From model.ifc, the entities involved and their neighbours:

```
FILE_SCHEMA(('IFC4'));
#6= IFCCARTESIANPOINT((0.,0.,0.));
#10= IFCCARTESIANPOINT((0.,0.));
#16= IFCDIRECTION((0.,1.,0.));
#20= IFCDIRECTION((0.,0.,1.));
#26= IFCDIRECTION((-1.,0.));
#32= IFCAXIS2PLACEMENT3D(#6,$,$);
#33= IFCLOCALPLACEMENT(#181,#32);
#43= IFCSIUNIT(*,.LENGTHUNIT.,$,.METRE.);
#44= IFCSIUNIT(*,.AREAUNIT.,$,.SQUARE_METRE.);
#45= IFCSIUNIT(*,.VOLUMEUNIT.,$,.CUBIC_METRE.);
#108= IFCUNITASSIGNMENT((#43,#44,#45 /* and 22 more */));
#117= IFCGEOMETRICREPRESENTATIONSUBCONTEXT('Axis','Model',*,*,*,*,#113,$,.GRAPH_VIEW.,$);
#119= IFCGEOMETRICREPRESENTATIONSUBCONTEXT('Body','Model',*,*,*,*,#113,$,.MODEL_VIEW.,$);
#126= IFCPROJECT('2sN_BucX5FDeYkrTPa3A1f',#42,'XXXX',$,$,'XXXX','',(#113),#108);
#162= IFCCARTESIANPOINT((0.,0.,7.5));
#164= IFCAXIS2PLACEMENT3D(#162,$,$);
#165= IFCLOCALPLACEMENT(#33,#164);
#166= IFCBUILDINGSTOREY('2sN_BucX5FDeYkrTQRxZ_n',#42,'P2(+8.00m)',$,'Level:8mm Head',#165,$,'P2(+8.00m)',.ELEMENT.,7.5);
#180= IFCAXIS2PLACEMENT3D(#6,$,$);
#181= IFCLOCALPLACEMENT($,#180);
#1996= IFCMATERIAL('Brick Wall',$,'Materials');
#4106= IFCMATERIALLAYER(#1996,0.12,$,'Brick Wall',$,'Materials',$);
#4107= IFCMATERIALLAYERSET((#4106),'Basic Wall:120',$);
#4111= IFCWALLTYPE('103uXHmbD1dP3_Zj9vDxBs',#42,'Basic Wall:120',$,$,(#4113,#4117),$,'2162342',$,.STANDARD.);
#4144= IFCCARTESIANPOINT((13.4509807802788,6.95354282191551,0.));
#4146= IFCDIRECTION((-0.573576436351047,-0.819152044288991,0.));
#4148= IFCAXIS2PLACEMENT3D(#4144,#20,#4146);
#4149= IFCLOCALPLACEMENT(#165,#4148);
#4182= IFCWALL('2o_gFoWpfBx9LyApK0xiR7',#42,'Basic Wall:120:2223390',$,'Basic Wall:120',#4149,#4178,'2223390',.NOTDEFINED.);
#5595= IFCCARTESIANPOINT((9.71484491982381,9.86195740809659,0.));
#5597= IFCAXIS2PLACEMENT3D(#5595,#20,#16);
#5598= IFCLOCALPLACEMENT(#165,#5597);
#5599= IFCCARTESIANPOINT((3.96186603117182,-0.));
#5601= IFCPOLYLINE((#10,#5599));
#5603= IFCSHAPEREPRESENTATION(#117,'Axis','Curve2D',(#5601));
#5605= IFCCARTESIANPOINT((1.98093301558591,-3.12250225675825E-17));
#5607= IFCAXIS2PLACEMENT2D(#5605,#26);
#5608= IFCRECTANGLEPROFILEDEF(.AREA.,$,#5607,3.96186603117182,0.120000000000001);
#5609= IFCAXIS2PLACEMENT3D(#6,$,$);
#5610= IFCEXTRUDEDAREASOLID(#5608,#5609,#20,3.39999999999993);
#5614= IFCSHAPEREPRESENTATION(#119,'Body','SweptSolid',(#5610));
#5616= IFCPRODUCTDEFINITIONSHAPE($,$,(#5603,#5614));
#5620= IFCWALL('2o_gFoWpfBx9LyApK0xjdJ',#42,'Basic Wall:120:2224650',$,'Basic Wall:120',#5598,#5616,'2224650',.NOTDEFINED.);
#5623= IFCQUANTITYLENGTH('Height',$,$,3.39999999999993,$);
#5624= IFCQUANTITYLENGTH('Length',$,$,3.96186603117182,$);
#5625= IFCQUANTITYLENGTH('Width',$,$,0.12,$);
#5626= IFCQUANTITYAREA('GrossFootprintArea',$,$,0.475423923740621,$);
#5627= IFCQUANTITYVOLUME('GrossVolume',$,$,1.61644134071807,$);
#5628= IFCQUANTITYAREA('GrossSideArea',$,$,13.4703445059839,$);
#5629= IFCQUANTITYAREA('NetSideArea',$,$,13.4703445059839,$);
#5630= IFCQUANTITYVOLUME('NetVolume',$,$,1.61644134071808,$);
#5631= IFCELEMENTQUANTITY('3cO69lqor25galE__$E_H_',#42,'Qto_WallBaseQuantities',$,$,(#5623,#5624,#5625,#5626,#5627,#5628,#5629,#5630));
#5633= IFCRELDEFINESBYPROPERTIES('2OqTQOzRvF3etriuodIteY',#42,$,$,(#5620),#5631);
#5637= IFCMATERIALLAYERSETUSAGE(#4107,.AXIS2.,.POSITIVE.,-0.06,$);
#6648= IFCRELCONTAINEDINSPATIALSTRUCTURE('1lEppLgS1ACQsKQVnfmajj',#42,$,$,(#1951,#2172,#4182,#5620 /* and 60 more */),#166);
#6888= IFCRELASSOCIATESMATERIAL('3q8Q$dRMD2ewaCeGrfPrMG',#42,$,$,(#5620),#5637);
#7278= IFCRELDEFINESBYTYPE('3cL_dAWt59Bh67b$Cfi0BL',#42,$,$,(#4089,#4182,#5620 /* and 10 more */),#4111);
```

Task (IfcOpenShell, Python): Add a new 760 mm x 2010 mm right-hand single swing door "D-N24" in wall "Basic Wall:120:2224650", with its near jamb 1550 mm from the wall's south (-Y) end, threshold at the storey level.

```python
import numpy as np
import ifcopenshell
import ifcopenshell.api.feature
import ifcopenshell.api.geometry
import ifcopenshell.api.pset
import ifcopenshell.api.root
import ifcopenshell.api.spatial
import ifcopenshell.geom
import ifcopenshell.util.element
import ifcopenshell.util.placement
import ifcopenshell.util.representation
import ifcopenshell.util.shape
import ifcopenshell.util.unit

model = ifcopenshell.open("model.ifc")
unit_scale = ifcopenshell.util.unit.calculate_unit_scale(model)
area_scale = ifcopenshell.util.unit.calculate_unit_scale(model, "AREAUNIT")
volume_scale = ifcopenshell.util.unit.calculate_unit_scale(model, "VOLUMEUNIT")
settings = ifcopenshell.geom.settings()


def volume(element):
    """Net volume in cubic metres, openings subtracted."""
    shape = ifcopenshell.geom.create_shape(settings, element)
    return ifcopenshell.util.shape.get_volume(shape.geometry)


wall = model.by_id(5620)
storey = ifcopenshell.util.element.get_container(wall, ifc_class="IfcBuildingStorey")
context = ifcopenshell.util.representation.get_context(model, "Model", "Body", "MODEL_VIEW")
before = volume(wall)

width, height, from_end, sill = 0.76, 2.01, 1.55, 0.0  # metres

# The wall runs along its own X axis, and the end named is its -X end.
wall_shape = ifcopenshell.geom.create_shape(settings, wall)
x, y, z = ifcopenshell.util.shape.get_vertices(wall_shape.geometry).T
start = x.min() + from_end
face, thickness = float(y.min()), float(y.max() - y.min())
wall_matrix = ifcopenshell.util.placement.get_local_placement(wall.ObjectPlacement)
level = ifcopenshell.util.placement.get_local_placement(storey.ObjectPlacement)[2, 3]


def in_wall(x, y):
    """Placement at x, y metres in the wall's axes, at sill height."""
    matrix = wall_matrix.copy()
    matrix[:, 3] = wall_matrix @ np.array([x / unit_scale, y / unit_scale, 0.0, 1.0])
    matrix[2, 3] = level + sill / unit_scale
    return matrix


# Opening: a box that overshoots both wall faces by 50 mm.
opening = ifcopenshell.api.root.create_entity(model, ifc_class="IfcOpeningElement", predefined_type="OPENING")
box = ifcopenshell.api.geometry.add_wall_representation(
    model, context=context, length=width, height=height, thickness=thickness + 0.1
)
ifcopenshell.api.geometry.assign_representation(model, product=opening, representation=box)
ifcopenshell.api.geometry.edit_object_placement(model, product=opening, matrix=in_wall(start, face - 0.05), is_si=False)
ifcopenshell.api.feature.add_feature(model, feature=opening, element=wall)

door = ifcopenshell.api.root.create_entity(model, ifc_class="IfcDoor", name="D-N24", predefined_type="DOOR")
door.OverallWidth, door.OverallHeight = width / unit_scale, height / unit_scale
door.OperationType = "SINGLE_SWING_RIGHT"
body = ifcopenshell.api.geometry.add_door_representation(
    model,
    context=context,
    overall_width=door.OverallWidth,
    overall_height=door.OverallHeight,
    operation_type="SINGLE_SWING_RIGHT",
    lining_properties={"LiningDepth": thickness / unit_scale, "ThresholdDepth": thickness / unit_scale},
)
ifcopenshell.api.geometry.assign_representation(model, product=door, representation=body)
ifcopenshell.api.spatial.assign_container(model, products=[door], relating_structure=storey)
ifcopenshell.api.feature.add_filling(model, opening=opening, element=door)

# The lining spans the wall, so the door starts at the wall face.
ifcopenshell.api.geometry.edit_object_placement(model, product=door, matrix=in_wall(start, face), is_si=False)

after = volume(wall)

# Update the wall's stored quantities.
qto = model.by_id(ifcopenshell.util.element.get_pset(wall, "Qto_WallBaseQuantities", should_inherit=False)["id"])
ifcopenshell.api.pset.edit_qto(model, qto=qto, properties={
    "NetSideArea": after / thickness / area_scale,
    "NetVolume": after / volume_scale,
})

print(f"wall volume {before:.3f} -> {after:.3f} m3")

model.write("model_v2.ifc")
```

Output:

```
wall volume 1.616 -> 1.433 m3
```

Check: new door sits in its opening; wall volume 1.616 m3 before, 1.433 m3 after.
